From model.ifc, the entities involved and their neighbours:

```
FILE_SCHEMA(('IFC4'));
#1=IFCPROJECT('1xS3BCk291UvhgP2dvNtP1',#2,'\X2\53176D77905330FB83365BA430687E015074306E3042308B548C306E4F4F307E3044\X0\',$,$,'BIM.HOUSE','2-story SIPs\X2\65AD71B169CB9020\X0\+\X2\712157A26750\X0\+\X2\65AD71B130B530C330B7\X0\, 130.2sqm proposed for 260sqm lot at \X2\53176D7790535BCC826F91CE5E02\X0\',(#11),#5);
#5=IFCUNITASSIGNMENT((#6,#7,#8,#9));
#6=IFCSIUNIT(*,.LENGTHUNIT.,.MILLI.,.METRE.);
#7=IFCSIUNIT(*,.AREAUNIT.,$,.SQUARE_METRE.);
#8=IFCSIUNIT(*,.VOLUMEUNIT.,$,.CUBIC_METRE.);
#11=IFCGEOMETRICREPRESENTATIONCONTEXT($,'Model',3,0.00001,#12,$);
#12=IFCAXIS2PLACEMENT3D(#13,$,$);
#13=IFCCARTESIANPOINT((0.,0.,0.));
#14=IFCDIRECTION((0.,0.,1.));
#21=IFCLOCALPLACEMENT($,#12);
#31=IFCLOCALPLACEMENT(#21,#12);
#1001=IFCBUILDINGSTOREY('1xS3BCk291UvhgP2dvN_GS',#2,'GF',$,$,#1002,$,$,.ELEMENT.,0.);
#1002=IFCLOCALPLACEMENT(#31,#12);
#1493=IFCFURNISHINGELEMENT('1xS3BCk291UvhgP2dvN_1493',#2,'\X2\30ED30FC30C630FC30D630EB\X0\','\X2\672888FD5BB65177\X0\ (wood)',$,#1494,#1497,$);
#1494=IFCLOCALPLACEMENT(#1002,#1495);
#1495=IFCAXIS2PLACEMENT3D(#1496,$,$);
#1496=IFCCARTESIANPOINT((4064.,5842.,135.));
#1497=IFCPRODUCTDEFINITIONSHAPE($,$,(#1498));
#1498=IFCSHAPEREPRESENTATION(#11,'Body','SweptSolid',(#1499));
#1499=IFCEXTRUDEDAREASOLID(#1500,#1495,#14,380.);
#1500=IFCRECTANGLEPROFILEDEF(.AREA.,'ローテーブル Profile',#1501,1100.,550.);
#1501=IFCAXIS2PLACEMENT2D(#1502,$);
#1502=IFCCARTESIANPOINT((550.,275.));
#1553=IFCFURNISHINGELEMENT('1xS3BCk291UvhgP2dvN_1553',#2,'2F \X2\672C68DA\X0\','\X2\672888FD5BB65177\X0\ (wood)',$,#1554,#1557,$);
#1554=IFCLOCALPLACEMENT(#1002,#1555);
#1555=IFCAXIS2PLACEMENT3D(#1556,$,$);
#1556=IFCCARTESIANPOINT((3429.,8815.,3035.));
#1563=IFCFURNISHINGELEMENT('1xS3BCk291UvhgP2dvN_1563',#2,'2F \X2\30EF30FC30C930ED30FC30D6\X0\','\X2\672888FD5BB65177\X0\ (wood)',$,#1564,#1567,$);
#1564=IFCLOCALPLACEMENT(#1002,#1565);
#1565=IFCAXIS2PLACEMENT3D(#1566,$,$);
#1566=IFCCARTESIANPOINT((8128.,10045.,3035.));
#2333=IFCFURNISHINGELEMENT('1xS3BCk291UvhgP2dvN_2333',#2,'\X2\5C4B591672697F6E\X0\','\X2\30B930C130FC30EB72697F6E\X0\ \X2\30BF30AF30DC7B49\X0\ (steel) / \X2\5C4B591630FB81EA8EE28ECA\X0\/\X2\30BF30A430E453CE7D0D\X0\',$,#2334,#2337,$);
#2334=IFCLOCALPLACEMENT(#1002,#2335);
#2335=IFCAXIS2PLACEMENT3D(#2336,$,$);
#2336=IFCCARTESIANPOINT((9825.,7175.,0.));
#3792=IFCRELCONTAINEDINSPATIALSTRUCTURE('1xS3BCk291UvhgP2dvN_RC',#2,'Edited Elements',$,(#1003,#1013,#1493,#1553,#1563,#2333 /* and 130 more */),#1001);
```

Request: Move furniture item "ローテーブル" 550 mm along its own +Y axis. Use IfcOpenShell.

```python
import ifcopenshell
import ifcopenshell.api.geometry
import ifcopenshell.util.placement
import ifcopenshell.util.unit

model = ifcopenshell.open("model.ifc")
unit_scale = ifcopenshell.util.unit.calculate_unit_scale(model)

item = model.by_id(1493)
matrix = ifcopenshell.util.placement.get_local_placement(item.ObjectPlacement)
matrix[:3, 3] += matrix[:3, 1] * 0.55 / unit_scale
ifcopenshell.api.geometry.edit_object_placement(model, product=item, matrix=matrix, is_si=False)

print(ifcopenshell.util.placement.get_local_placement(item.ObjectPlacement).round(3) + 0.0)

model.write("model_edited.ifc")
```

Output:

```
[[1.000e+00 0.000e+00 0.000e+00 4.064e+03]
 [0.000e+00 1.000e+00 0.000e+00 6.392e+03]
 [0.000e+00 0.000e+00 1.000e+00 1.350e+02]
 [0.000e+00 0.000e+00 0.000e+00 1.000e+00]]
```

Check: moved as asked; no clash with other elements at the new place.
